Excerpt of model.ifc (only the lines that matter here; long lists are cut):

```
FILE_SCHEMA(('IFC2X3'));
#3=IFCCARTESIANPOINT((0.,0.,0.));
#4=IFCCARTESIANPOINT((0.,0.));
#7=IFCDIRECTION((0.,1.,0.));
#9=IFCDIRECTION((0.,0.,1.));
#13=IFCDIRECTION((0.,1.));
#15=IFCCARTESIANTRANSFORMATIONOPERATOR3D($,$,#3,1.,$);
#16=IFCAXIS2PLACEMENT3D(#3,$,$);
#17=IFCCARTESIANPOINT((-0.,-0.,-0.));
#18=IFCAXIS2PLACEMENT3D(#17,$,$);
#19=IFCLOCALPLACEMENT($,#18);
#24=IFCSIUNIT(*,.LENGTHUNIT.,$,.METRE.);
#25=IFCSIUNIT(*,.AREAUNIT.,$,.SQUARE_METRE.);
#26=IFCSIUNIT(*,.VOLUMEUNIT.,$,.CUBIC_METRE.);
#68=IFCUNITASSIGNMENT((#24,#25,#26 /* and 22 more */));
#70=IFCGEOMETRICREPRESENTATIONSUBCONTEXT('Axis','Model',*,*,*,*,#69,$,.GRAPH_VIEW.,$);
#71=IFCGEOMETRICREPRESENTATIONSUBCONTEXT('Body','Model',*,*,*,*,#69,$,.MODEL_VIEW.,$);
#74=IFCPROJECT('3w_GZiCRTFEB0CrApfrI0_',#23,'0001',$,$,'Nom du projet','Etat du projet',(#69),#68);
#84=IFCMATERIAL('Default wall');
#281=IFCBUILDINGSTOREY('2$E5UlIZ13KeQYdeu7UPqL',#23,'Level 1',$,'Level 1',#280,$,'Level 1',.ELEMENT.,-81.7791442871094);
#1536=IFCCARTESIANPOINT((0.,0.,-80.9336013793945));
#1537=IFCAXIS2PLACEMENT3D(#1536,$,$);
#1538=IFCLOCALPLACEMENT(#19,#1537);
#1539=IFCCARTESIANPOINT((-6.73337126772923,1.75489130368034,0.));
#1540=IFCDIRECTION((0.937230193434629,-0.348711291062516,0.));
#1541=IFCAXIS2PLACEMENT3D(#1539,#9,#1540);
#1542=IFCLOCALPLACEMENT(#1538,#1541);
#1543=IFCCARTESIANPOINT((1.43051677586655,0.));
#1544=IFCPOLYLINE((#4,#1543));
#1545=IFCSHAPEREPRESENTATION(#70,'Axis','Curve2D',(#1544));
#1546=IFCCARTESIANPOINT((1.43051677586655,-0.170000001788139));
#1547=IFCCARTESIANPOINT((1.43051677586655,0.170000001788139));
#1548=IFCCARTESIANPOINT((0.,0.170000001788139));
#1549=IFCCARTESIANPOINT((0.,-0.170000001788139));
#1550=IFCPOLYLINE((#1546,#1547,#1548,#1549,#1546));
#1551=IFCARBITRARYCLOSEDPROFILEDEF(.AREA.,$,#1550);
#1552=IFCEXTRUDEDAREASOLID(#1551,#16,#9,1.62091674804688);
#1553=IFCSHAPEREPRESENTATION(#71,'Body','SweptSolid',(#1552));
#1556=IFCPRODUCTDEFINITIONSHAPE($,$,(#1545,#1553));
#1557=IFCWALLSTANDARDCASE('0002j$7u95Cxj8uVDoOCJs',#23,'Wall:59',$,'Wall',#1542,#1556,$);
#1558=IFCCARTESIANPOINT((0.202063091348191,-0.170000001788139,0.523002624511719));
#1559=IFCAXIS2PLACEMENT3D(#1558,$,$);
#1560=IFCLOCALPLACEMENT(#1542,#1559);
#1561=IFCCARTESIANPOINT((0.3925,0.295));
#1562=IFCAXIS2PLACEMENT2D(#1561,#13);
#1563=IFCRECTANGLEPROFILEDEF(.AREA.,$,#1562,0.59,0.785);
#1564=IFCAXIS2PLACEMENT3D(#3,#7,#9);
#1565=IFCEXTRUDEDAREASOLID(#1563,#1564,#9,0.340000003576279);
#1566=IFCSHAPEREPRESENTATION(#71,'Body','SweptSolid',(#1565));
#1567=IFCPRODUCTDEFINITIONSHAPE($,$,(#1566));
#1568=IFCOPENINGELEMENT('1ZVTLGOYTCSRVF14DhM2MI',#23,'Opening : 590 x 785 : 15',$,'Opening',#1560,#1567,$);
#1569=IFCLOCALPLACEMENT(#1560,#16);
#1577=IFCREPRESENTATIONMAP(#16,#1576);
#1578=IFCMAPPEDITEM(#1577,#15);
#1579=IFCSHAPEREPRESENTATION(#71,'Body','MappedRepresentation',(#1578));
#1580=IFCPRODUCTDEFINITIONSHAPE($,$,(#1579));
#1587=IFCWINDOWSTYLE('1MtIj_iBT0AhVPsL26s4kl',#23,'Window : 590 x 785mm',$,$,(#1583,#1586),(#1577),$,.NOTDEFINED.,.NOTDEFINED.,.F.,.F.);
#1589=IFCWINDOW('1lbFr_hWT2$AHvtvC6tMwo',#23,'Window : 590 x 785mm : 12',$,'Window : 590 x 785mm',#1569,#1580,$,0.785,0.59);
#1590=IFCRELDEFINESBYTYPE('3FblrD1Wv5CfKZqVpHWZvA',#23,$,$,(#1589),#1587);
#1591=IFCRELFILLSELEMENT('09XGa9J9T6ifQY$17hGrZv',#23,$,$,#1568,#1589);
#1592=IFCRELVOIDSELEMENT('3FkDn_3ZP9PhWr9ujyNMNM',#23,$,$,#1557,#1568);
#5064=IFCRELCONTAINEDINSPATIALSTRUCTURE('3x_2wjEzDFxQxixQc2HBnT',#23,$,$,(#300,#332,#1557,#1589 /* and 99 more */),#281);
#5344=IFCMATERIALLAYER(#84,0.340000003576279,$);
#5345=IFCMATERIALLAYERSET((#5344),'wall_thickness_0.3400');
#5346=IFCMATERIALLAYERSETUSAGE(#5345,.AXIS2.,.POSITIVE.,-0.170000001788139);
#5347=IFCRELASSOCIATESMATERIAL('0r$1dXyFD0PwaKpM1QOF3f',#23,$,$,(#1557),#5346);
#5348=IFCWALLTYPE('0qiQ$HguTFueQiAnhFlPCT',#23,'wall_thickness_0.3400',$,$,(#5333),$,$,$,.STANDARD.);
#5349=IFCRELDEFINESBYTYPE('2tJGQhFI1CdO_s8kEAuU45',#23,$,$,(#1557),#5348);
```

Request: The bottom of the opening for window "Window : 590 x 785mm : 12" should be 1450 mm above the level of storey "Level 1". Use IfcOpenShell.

```python
import numpy as np
import ifcopenshell
import ifcopenshell.api.geometry
import ifcopenshell.geom
import ifcopenshell.util.element
import ifcopenshell.util.placement
import ifcopenshell.util.shape
import ifcopenshell.util.unit

model = ifcopenshell.open("model.ifc")
unit_scale = ifcopenshell.util.unit.calculate_unit_scale(model)

window = model.by_guid("1lbFr_hWT2$AHvtvC6tMwo")
opening = window.FillsVoids[0].RelatingOpeningElement
storey = ifcopenshell.util.element.get_container(window, ifc_class="IfcBuildingStorey")
level = ifcopenshell.util.placement.get_local_placement(storey.ObjectPlacement)[2, 3]

# The opening's origin need not be at the sill, so measure its lowest point.
shape = ifcopenshell.geom.create_shape(ifcopenshell.geom.settings(), opening)
bottom = ifcopenshell.util.shape.get_shape_bottom_elevation(shape, shape.geometry) / unit_scale
dz = level + 1.45 - bottom

shift = np.array([0.0, 0.0, dz])
# The window is placed relative to its opening, so it follows when the opening moves.
matrix = ifcopenshell.util.placement.get_local_placement(opening.ObjectPlacement)
matrix[:3, 3] += shift
ifcopenshell.api.geometry.edit_object_placement(
    model, product=opening, matrix=matrix, is_si=False, should_transform_children=True
)

print(f"moved by {dz * unit_scale:+.3f} m")

model.write("model_updated.ifc")
```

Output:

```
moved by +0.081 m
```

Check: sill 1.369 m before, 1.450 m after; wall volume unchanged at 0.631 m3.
